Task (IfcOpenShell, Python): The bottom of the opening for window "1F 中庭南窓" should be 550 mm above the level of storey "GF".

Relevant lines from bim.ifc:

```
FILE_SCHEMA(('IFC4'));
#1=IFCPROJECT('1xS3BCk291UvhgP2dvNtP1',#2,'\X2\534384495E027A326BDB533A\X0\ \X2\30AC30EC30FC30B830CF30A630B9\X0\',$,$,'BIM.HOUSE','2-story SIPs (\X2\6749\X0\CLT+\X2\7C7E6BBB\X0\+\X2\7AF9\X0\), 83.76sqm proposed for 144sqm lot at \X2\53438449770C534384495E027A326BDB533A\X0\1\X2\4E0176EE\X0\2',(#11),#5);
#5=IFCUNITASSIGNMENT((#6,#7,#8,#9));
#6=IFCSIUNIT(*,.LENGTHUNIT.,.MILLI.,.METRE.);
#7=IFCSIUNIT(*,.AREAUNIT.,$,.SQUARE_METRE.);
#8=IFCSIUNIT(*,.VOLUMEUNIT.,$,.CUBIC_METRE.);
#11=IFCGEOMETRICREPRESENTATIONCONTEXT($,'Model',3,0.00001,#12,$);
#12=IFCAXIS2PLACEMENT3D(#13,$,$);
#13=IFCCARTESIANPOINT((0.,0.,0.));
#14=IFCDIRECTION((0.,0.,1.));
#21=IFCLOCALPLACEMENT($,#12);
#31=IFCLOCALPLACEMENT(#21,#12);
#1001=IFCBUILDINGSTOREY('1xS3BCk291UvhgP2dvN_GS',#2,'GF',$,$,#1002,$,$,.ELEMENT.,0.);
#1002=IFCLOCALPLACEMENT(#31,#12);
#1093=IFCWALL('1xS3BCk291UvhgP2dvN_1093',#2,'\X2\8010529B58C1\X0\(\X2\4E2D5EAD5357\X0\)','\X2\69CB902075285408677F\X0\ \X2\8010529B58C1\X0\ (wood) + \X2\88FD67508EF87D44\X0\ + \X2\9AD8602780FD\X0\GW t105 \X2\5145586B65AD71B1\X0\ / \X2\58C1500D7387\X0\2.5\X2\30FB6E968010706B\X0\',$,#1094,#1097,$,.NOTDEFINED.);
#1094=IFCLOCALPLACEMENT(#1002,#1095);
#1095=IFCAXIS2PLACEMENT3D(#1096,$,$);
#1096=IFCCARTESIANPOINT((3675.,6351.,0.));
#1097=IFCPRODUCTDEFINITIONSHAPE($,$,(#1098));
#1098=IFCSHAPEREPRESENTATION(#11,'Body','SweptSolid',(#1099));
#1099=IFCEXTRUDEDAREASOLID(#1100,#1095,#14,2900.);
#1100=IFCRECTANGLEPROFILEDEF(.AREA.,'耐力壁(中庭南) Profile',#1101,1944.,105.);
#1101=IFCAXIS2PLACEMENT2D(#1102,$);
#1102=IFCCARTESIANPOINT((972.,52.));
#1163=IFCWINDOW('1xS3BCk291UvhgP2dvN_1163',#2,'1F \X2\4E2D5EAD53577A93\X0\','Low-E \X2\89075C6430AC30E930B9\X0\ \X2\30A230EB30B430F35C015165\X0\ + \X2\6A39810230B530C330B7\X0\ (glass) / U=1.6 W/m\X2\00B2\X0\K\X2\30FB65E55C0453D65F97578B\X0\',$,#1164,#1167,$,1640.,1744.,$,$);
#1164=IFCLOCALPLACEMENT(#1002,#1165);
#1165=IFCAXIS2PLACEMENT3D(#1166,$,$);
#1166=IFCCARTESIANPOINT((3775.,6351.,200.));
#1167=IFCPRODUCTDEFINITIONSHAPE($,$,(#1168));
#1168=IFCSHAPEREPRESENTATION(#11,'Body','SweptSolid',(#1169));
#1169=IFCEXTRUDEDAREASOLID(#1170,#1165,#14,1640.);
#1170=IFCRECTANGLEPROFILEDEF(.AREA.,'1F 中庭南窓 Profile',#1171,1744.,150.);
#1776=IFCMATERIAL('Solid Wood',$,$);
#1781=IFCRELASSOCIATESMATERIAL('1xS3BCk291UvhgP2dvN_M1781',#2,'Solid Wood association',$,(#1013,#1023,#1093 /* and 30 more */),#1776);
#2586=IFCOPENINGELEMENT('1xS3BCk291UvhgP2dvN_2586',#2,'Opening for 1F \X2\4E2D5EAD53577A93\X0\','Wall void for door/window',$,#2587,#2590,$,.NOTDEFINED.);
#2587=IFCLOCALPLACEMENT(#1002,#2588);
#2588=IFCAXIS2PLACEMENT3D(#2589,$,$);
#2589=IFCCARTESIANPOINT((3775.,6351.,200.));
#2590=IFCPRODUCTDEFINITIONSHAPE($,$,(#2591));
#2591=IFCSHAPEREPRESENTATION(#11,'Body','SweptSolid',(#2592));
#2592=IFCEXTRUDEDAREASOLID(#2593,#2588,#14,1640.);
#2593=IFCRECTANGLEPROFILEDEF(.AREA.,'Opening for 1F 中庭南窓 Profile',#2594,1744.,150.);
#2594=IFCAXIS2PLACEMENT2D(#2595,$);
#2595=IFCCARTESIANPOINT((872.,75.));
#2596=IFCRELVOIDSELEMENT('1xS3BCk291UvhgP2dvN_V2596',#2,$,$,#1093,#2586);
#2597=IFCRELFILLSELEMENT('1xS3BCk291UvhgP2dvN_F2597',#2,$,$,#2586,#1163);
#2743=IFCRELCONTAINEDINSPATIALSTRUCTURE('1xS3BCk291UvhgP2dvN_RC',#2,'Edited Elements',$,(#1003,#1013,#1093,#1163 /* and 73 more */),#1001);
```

```python
import numpy as np
import ifcopenshell
import ifcopenshell.api.geometry
import ifcopenshell.geom
import ifcopenshell.util.element
import ifcopenshell.util.placement
import ifcopenshell.util.shape
import ifcopenshell.util.unit

model = ifcopenshell.open("bim.ifc")
unit_scale = ifcopenshell.util.unit.calculate_unit_scale(model)

window = model.by_id(1163)
opening = window.FillsVoids[0].RelatingOpeningElement
storey = ifcopenshell.util.element.get_container(window, ifc_class="IfcBuildingStorey")
level = ifcopenshell.util.placement.get_local_placement(storey.ObjectPlacement)[2, 3]

# The opening's origin need not be at the sill, so measure its lowest point.
shape = ifcopenshell.geom.create_shape(ifcopenshell.geom.settings(), opening)
bottom = ifcopenshell.util.shape.get_shape_bottom_elevation(shape, shape.geometry) / unit_scale
dz = level + 550.0 - bottom

shift = np.array([0.0, 0.0, dz])
# The window is not placed relative to its opening, so move both.
for product in (opening, window):
    matrix = ifcopenshell.util.placement.get_local_placement(product.ObjectPlacement)
    matrix[:3, 3] += shift
    ifcopenshell.api.geometry.edit_object_placement(model, product=product, matrix=matrix, is_si=False)

print(f"moved by {dz * unit_scale:+.3f} m")

model.write("bim_updated.ifc")
```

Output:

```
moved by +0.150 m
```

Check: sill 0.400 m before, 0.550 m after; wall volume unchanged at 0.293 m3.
